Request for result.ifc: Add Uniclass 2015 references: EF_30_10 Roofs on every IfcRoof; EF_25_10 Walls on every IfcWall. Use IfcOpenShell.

First a look at what the model holds.

```python
import ifcopenshell

model = ifcopenshell.open("result.ifc")
print(model.schema)
print("classifications:", [c.Name for c in model.by_type("IfcClassification")])
for ifc_class in ("IfcDoor", "IfcRoof", "IfcStair", "IfcWall", "IfcWindow"):
    print(ifc_class, len(model.by_type(ifc_class)))
```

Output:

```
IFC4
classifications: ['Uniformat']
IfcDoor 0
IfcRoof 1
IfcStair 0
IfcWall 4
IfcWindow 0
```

```python
import ifcopenshell
import ifcopenshell.api.classification

model = ifcopenshell.open("result.ifc")

system = ifcopenshell.api.classification.add_classification(model, classification="Uniclass 2015")

codes = {
    "IfcRoof": ("EF_30_10", "Roofs"),
    "IfcWall": ("EF_25_10", "Walls"),
}
for ifc_class, (code, name) in codes.items():
    products = model.by_type(ifc_class)
    ifcopenshell.api.classification.add_reference(
        model, products=products, classification=system, identification=code, name=name
    )
    print(code, len(products))

model.write("result-out.ifc")
```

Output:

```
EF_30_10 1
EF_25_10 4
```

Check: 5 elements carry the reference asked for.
